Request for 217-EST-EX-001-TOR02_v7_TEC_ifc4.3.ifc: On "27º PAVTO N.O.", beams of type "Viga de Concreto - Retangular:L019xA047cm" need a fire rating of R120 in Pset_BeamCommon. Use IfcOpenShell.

First a look at what the model holds.

```python
import ifcopenshell
import ifcopenshell.util.element

model = ifcopenshell.open("217-EST-EX-001-TOR02_v7_TEC_ifc4.3.ifc")
print(model.schema)
storey = next(s for s in model.by_type("IfcBuildingStorey") if s.Name == "27º PAVTO N.O.")
beams = [e for e in ifcopenshell.util.element.get_decomposition(storey) if e.is_a("IfcBeam")]
seen = {}
for e in beams:
    element_type = ifcopenshell.util.element.get_type(e)
    key = (element_type.Name if element_type != e and element_type else None, ifcopenshell.util.element.get_pset(e, "Pset_BeamCommon", "FireRating"))
    seen[key] = seen.get(key, 0) + 1
for (name, value), count in sorted(seen.items(), key=str):
    print(count, "x", name, "|", value)
```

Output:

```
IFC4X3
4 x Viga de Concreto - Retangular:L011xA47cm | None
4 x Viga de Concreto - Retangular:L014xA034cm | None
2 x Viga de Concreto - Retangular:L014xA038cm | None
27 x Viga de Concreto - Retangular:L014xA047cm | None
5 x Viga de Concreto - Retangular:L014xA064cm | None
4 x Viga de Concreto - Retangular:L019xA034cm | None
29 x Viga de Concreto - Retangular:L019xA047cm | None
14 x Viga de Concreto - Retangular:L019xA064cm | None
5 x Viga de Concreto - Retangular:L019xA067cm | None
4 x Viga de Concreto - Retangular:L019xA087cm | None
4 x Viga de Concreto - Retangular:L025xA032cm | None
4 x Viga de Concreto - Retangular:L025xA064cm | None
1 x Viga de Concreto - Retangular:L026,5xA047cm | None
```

```python
import ifcopenshell
import ifcopenshell.api.pset
import ifcopenshell.util.element

model = ifcopenshell.open("217-EST-EX-001-TOR02_v7_TEC_ifc4.3.ifc")

storey = next(s for s in model.by_type("IfcBuildingStorey") if s.Name == "27º PAVTO N.O.")
beams = [e for e in ifcopenshell.util.element.get_decomposition(storey) if e.is_a("IfcBeam")]

count = 0
for e in beams:
    element_type = ifcopenshell.util.element.get_type(e)
    if element_type in (None, e) or element_type.Name != "Viga de Concreto - Retangular:L019xA047cm":
        continue
    # add_pset returns the element's existing set when there is one.
    pset = ifcopenshell.api.pset.add_pset(model, product=e, name="Pset_BeamCommon")
    ifcopenshell.api.pset.edit_pset(model, pset=pset, properties={"FireRating": "R120"})
    count += 1

print(count, "beams updated")

model.write("217-EST-EX-001-TOR02_v7_TEC_ifc4.3_updated.ifc")
```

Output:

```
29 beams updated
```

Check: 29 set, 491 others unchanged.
